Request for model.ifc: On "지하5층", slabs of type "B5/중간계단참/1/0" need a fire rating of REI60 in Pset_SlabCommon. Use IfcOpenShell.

First a look at what the model holds.

```python
import ifcopenshell
import ifcopenshell.util.element

model = ifcopenshell.open("model.ifc")
print(model.schema)
storey = next(s for s in model.by_type("IfcBuildingStorey") if s.Name == "지하5층")
slabs = [e for e in ifcopenshell.util.element.get_decomposition(storey) if e.is_a("IfcSlab")]
seen = {}
for e in slabs:
    element_type = ifcopenshell.util.element.get_type(e)
    key = (element_type.Name if element_type != e and element_type else None, ifcopenshell.util.element.get_pset(e, "Pset_SlabCommon", "FireRating"))
    seen[key] = seen.get(key, 0) + 1
for (name, value), count in sorted(seen.items(), key=str):
    print(count, "x", name, "|", value)
```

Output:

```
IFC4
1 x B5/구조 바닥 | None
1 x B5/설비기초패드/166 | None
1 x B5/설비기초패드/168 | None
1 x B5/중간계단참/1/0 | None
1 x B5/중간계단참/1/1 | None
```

```python
import ifcopenshell
import ifcopenshell.api.pset
import ifcopenshell.util.element

model = ifcopenshell.open("model.ifc")

storey = next(s for s in model.by_type("IfcBuildingStorey") if s.Name == "지하5층")
slabs = [e for e in ifcopenshell.util.element.get_decomposition(storey) if e.is_a("IfcSlab")]

count = 0
for e in slabs:
    element_type = ifcopenshell.util.element.get_type(e)
    if element_type in (None, e) or element_type.Name != "B5/중간계단참/1/0":
        continue
    # add_pset returns the element's existing set when there is one.
    pset = ifcopenshell.api.pset.add_pset(model, product=e, name="Pset_SlabCommon")
    ifcopenshell.api.pset.edit_pset(model, pset=pset, properties={"FireRating": "REI60"})
    count += 1

print(count, "slabs updated")

model.write("model_updated.ifc")
```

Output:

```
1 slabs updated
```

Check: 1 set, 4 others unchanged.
